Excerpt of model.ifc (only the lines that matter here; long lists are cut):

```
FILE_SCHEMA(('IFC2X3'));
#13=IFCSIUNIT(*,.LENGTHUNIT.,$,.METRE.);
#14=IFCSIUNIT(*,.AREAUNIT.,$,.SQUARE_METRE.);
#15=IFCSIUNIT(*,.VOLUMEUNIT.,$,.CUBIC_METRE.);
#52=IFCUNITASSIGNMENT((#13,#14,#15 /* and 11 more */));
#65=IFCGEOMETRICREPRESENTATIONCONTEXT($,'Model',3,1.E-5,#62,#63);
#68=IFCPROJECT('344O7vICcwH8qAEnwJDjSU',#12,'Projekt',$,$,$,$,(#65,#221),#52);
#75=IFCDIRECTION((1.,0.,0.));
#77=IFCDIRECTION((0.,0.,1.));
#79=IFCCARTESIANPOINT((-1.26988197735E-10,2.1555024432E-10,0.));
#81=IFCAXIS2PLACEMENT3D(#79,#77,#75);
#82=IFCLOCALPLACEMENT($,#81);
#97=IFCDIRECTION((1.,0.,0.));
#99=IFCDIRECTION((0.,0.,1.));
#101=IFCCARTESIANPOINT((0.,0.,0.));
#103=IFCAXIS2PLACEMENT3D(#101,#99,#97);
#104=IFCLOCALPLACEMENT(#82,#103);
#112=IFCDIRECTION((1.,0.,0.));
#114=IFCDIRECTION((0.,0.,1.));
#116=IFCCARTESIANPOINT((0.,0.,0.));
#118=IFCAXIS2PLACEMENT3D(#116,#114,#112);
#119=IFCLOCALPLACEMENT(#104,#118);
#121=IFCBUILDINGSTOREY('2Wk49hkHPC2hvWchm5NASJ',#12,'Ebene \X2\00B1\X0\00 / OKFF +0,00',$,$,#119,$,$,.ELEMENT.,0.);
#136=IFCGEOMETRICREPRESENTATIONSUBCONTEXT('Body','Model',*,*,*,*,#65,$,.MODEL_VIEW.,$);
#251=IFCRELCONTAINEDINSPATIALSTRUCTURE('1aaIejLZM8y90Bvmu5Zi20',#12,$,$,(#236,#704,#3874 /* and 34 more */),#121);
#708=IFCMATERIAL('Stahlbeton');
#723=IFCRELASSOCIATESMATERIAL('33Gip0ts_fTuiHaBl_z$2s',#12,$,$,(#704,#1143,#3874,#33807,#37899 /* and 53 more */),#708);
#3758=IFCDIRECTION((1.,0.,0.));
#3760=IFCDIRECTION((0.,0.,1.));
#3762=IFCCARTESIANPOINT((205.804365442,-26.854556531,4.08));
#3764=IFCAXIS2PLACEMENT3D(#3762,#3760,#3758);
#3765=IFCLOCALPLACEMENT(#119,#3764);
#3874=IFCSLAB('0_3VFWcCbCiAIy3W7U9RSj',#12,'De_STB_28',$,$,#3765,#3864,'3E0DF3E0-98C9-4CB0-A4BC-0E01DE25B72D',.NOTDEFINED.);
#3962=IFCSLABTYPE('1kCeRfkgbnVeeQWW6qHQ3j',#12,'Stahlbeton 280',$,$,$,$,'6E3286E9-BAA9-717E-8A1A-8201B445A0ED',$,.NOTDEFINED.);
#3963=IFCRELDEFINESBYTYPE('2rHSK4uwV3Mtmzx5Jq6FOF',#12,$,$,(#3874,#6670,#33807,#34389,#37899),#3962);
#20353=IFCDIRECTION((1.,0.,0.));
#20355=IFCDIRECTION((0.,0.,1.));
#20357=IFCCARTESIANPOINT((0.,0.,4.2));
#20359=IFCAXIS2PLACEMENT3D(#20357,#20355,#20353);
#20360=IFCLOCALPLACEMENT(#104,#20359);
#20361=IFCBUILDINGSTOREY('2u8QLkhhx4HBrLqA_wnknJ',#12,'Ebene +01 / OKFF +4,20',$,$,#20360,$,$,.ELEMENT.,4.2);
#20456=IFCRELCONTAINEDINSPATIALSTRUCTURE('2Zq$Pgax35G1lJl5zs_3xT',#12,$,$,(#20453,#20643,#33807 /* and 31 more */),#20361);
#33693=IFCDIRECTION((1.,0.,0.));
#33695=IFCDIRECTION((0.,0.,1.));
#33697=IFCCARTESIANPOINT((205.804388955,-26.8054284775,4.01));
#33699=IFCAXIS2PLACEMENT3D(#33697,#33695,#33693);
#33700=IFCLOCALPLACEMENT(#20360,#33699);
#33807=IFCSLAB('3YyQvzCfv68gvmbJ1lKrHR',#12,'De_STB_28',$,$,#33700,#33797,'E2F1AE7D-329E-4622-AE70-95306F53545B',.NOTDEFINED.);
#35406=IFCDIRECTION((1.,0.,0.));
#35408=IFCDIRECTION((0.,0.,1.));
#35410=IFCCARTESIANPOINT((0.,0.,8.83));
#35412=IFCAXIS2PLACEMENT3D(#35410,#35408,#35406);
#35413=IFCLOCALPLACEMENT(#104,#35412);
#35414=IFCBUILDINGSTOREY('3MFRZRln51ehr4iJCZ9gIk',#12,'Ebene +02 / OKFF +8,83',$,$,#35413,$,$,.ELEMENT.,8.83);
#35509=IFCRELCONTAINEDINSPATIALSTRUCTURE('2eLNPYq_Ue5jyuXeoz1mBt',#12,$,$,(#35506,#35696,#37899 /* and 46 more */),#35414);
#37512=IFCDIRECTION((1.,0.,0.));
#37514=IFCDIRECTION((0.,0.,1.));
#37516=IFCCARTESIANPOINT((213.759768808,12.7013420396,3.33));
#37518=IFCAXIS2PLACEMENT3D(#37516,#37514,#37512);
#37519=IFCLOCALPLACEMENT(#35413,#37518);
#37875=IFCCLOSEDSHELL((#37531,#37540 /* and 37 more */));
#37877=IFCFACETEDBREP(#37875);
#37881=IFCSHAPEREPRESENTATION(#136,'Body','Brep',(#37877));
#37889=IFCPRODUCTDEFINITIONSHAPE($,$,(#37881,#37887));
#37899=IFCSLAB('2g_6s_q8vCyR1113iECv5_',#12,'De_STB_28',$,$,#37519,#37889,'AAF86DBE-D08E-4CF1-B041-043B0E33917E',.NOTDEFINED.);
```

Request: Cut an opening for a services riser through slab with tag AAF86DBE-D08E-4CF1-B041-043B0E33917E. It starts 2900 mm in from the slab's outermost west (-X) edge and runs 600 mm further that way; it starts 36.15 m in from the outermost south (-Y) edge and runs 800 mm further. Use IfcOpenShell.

```python
import numpy as np
import ifcopenshell
import ifcopenshell.api.feature
import ifcopenshell.api.geometry
import ifcopenshell.api.root
import ifcopenshell.geom
import ifcopenshell.util.placement
import ifcopenshell.util.representation
import ifcopenshell.util.shape
import ifcopenshell.util.unit

model = ifcopenshell.open("model.ifc")
unit_scale = ifcopenshell.util.unit.calculate_unit_scale(model)
settings = ifcopenshell.geom.settings()


def volume(element):
    """Net volume in cubic metres, openings subtracted."""
    shape = ifcopenshell.geom.create_shape(settings, element)
    return ifcopenshell.util.shape.get_volume(shape.geometry)


slab = model.by_guid("2g_6s_q8vCyR1113iECv5_")
before = volume(slab)

# Extent in the slab's own axes, in metres. The edges named are its -X and -Y sides.
slab_shape = ifcopenshell.geom.create_shape(settings, slab)
vertices = ifcopenshell.util.shape.get_vertices(slab_shape.geometry)
x_min, y_min, bottom = vertices.min(axis=0)
top = vertices[:, 2].max()

opening = ifcopenshell.api.root.create_entity(model, ifc_class="IfcOpeningElement", name="Services riser opening")
context = ifcopenshell.util.representation.get_context(model, "Model", "Body", "MODEL_VIEW")
width, depth = 0.6, 0.8
outline = [(0.0, 0.0), (width, 0.0), (width, depth), (0.0, depth), (0.0, 0.0)]
# Overshoot both faces by 50 mm so the cut is clean.
shape = ifcopenshell.api.geometry.add_slab_representation(
    model, context=context, depth=top - bottom + 0.1, polyline=outline
)
ifcopenshell.api.geometry.assign_representation(model, product=opening, representation=shape)

matrix = ifcopenshell.util.placement.get_local_placement(slab.ObjectPlacement)
matrix[:, 3] = matrix @ np.append(np.array([x_min + 2.9, y_min + 36.15, bottom - 0.05]) / unit_scale, 1.0)
ifcopenshell.api.geometry.edit_object_placement(model, product=opening, matrix=matrix, is_si=False)
ifcopenshell.api.feature.add_feature(model, feature=opening, element=slab)

after = volume(slab)

print(f"slab volume {before:.3f} -> {after:.3f} m3")

model.write("model_rev.ifc")
```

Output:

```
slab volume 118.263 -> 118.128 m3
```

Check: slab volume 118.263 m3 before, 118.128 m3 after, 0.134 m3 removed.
